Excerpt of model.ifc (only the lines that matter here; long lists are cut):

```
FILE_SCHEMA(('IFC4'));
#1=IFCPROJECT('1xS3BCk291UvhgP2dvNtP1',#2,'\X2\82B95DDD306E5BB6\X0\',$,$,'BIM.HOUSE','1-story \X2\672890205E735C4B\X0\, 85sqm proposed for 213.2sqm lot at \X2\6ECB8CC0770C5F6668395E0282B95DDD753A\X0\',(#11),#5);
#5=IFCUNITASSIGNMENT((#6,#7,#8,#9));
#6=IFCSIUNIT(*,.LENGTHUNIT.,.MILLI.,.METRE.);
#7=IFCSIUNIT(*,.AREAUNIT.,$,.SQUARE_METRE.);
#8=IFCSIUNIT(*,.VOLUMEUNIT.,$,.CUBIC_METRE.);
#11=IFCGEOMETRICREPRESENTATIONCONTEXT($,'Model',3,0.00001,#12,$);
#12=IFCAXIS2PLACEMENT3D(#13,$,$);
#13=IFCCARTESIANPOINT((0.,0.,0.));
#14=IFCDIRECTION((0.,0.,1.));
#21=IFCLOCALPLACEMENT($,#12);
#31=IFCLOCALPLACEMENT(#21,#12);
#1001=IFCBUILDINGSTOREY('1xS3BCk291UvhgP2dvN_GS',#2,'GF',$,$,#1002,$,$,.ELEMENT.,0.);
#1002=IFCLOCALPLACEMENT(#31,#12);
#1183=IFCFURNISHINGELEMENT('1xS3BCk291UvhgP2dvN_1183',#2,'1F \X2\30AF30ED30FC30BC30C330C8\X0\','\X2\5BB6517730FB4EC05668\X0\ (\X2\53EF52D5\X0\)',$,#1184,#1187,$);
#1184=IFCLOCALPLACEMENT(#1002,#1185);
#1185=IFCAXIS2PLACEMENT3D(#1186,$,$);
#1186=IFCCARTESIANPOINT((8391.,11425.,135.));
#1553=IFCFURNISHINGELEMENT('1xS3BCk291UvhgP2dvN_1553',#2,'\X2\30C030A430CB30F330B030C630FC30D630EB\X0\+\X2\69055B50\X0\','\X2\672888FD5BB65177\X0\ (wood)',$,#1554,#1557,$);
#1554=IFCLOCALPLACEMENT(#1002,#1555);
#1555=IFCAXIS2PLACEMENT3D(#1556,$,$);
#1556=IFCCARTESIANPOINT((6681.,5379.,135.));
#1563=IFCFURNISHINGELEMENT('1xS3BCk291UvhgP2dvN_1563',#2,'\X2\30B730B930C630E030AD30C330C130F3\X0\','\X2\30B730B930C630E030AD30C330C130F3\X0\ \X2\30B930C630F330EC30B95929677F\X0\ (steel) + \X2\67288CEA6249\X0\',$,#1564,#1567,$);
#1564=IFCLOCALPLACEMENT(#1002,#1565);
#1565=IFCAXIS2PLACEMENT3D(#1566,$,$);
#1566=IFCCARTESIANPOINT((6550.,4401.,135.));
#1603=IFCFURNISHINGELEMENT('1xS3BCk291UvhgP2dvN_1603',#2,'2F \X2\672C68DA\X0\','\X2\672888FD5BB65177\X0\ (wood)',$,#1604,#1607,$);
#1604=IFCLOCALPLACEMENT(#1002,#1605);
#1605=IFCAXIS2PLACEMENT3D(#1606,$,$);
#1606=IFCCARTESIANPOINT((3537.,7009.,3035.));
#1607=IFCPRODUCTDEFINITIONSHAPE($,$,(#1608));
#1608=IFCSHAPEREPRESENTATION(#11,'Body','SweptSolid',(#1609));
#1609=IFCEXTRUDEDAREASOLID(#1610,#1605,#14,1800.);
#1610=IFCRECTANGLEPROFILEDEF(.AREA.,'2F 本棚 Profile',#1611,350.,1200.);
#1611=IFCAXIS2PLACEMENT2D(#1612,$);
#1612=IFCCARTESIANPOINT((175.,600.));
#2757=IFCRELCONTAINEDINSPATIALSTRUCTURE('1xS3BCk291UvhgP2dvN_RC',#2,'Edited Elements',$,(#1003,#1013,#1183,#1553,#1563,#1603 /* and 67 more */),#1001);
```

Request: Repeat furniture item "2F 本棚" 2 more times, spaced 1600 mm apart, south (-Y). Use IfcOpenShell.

```python
import numpy as np
import ifcopenshell
import ifcopenshell.api.geometry
import ifcopenshell.api.root
import ifcopenshell.util.element
import ifcopenshell.util.placement

model = ifcopenshell.open("model.ifc")


def reuse_history(source, copy):
    """copy_class also copies each property set's owner history, people and application; keep the originals."""
    for rel in copy.IsDefinedBy:
        if rel.is_a("IfcRelDefinesByProperties") and (history := rel.RelatingPropertyDefinition.OwnerHistory):
            rel.RelatingPropertyDefinition.OwnerHistory = source.OwnerHistory
            ifcopenshell.util.element.remove_deep2(model, history)


source = model.by_guid("1xS3BCk291UvhgP2dvN_1603")
base = ifcopenshell.util.placement.get_local_placement(source.ObjectPlacement)
step = np.array([0.0, -1.0, 0.0]) * 1600.0

for i in range(1, 3):
    copy = ifcopenshell.api.root.copy_class(model, product=source)
    copy.Representation = ifcopenshell.util.element.copy_deep(
        model, source.Representation, exclude=["IfcGeometricRepresentationContext", "IfcRepresentationMap"]
    )
    reuse_history(source, copy)
    matrix = base.copy()
    matrix[:3, 3] += i * step
    print("added at", matrix[:3, 3].round(3) + 0.0)
    ifcopenshell.api.geometry.edit_object_placement(model, product=copy, matrix=matrix, is_si=False)

model.write("model_rev.ifc")
```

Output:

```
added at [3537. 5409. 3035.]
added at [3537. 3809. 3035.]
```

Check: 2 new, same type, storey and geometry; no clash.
